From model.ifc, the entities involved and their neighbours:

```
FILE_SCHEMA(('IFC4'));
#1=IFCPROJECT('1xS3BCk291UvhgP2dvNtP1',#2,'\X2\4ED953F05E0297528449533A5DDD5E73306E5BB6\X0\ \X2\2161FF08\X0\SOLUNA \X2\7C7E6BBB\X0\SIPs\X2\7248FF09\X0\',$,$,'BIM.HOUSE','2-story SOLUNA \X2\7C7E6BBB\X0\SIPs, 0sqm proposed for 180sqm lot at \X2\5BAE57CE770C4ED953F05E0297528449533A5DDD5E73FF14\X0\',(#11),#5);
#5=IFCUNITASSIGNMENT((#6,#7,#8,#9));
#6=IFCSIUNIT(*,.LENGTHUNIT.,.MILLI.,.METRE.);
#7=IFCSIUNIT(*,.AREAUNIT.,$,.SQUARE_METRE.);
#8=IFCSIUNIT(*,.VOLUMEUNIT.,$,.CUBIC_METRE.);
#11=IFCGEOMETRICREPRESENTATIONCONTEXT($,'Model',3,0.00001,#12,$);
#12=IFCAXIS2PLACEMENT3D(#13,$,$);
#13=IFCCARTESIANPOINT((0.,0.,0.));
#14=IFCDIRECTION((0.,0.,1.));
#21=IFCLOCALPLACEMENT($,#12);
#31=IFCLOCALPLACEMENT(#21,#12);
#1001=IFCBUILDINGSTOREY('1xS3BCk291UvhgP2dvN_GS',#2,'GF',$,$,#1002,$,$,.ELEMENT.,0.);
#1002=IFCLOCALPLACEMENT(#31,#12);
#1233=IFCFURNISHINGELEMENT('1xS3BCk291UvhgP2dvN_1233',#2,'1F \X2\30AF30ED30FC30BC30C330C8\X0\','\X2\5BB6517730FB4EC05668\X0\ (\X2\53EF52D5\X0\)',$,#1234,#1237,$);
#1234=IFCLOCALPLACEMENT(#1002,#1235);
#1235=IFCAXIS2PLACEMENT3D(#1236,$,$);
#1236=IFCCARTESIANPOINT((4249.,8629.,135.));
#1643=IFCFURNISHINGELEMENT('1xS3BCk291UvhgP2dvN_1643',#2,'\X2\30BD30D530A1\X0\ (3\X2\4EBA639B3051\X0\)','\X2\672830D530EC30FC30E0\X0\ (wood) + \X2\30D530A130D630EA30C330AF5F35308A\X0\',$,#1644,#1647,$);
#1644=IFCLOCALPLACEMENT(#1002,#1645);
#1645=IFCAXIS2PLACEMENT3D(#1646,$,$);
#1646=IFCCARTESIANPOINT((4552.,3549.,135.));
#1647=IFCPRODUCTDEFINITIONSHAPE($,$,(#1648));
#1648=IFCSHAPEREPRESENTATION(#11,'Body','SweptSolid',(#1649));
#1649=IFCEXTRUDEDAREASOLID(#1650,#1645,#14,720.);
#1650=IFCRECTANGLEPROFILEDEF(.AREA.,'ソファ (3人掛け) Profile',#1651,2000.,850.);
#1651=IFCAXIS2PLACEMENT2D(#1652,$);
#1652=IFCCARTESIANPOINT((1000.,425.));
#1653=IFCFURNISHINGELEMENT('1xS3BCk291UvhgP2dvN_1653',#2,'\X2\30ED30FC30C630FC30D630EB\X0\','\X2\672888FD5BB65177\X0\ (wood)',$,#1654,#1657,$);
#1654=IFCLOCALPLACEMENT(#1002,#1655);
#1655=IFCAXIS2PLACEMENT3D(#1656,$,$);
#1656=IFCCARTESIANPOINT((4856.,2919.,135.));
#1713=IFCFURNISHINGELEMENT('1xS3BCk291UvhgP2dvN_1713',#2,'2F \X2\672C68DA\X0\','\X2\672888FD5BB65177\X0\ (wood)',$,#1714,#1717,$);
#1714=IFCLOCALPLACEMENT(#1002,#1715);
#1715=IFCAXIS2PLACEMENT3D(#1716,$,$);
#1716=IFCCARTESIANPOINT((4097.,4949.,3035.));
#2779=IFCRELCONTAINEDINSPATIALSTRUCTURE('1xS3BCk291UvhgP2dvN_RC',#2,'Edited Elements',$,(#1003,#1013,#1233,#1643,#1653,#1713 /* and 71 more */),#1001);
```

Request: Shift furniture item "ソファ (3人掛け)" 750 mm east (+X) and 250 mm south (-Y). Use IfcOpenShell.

```python
import ifcopenshell
import ifcopenshell.api.geometry
import ifcopenshell.util.placement

model = ifcopenshell.open("model.ifc")

item = model.by_guid("1xS3BCk291UvhgP2dvN_1643")
matrix = ifcopenshell.util.placement.get_local_placement(item.ObjectPlacement)
matrix[0, 3] += 750.0
matrix[1, 3] -= 250.0
ifcopenshell.api.geometry.edit_object_placement(model, product=item, matrix=matrix, is_si=False)

print(ifcopenshell.util.placement.get_local_placement(item.ObjectPlacement).round(3) + 0.0)

model.write("model_updated.ifc")
```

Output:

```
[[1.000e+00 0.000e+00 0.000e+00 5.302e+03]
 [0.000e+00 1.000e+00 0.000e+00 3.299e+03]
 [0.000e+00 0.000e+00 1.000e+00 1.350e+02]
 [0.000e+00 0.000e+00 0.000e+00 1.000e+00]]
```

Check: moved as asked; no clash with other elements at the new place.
